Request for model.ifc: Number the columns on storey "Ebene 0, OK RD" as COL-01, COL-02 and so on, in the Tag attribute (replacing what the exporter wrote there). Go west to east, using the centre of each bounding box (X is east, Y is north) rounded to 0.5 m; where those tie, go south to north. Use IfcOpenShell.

First a look at what the model holds.

```python
import ifcopenshell
import ifcopenshell.util.element
import ifcopenshell.util.placement

model = ifcopenshell.open("model.ifc")
print(model.schema)
storey = next(s for s in model.by_type("IfcBuildingStorey") if s.Name == "Ebene 0, OK RD")
columns = [e for e in ifcopenshell.util.element.get_decomposition(storey) if e.is_a("IfcColumn")]
for e in sorted(columns, key=lambda e: e.id()):
    origin = ifcopenshell.util.placement.get_local_placement(e.ObjectPlacement)[:3, 3]
    print(e.id(), e.Tag, e.Name, origin.round(2) + 0.0, sep=" | ")
```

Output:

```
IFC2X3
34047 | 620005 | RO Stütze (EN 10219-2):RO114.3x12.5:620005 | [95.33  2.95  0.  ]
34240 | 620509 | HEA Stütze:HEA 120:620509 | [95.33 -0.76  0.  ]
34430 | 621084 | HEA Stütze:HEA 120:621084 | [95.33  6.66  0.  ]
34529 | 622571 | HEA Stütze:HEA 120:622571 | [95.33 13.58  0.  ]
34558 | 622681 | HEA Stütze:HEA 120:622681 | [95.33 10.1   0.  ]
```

```python
import ifcopenshell
import ifcopenshell.geom
import ifcopenshell.util.element
import ifcopenshell.util.shape

model = ifcopenshell.open("model.ifc")
settings = ifcopenshell.geom.settings()
settings.set("use-world-coords", True)


def centre(element):
    shape = ifcopenshell.geom.create_shape(settings, element)
    return ifcopenshell.util.shape.get_bbox_centroid(shape.geometry)


storey = next(s for s in model.by_type("IfcBuildingStorey") if s.Name == "Ebene 0, OK RD")
columns = [e for e in ifcopenshell.util.element.get_decomposition(storey) if e.is_a("IfcColumn")]

# Insertion points can sit at a corner or the storey origin, so sort by the geometry (in metres).
centres = {e: centre(e) for e in columns}
columns.sort(key=lambda e: (round(centres[e][0] / 0.5), centres[e][1]))

for i, e in enumerate(columns, start=1):
    number = f"COL-{i:02d}"
    e.Tag = number
    print(e.id(), number)

model.write("model_rev.ifc")
```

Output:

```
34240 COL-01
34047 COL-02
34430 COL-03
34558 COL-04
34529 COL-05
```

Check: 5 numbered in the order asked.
